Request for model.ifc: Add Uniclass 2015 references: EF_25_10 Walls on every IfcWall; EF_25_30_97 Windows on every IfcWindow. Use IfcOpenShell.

First a look at what the model holds.

```python
import ifcopenshell

model = ifcopenshell.open("model.ifc")
print(model.schema)
print("classifications:", [c.Name for c in model.by_type("IfcClassification")])
for ifc_class in ("IfcDoor", "IfcRoof", "IfcStair", "IfcWall", "IfcWindow"):
    print(ifc_class, len(model.by_type(ifc_class)))
```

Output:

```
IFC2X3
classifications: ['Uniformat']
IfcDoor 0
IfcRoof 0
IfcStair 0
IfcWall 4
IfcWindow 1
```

```python
import ifcopenshell
import ifcopenshell.api.classification

model = ifcopenshell.open("model.ifc")

# IFC2X3 requires Source and Edition and has no link from the project to the system.
system = model.create_entity("IfcClassification", Source="NBS", Edition="2015", Name="Uniclass 2015")

codes = {
    "IfcWall": ("EF_25_10", "Walls"),
    "IfcWindow": ("EF_25_30_97", "Windows"),
}
for ifc_class, (code, name) in codes.items():
    products = model.by_type(ifc_class)
    ifcopenshell.api.classification.add_reference(
        model, products=products, classification=system, identification=code, name=name
    )
    print(code, len(products))

model.write("model_edited.ifc")
```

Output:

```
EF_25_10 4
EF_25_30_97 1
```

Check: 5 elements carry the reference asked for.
